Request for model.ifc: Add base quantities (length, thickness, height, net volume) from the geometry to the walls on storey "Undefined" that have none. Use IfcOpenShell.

First a look at what the model holds.

```python
import ifcopenshell
import ifcopenshell.util.element
import ifcopenshell.util.unit

model = ifcopenshell.open("model.ifc")
print(model.schema)
for unit_type in ("LENGTHUNIT", "AREAUNIT", "VOLUMEUNIT"):
    print(unit_type, ifcopenshell.util.unit.calculate_unit_scale(model, unit_type))
storey = next(s for s in model.by_type("IfcBuildingStorey") if s.Name == "Undefined")
walls = [e for e in ifcopenshell.util.element.get_decomposition(storey) if e.is_a("IfcWall")]
for e in sorted(walls, key=lambda e: e.id()):
    print(e.id(), e.is_a(), e.Name, list(ifcopenshell.util.element.get_psets(e, qtos_only=True)), sep=" | ")
```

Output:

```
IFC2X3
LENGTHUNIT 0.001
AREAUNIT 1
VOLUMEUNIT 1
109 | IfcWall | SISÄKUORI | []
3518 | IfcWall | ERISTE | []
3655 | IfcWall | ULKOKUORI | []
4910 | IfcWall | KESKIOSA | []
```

```python
import ifcopenshell
import ifcopenshell.api.pset
import ifcopenshell.geom
import ifcopenshell.util.element
import ifcopenshell.util.shape
import ifcopenshell.util.unit

model = ifcopenshell.open("model.ifc")
unit_scale = ifcopenshell.util.unit.calculate_unit_scale(model)
volume_scale = ifcopenshell.util.unit.calculate_unit_scale(model, "VOLUMEUNIT")
settings = ifcopenshell.geom.settings()

storey = next(s for s in model.by_type("IfcBuildingStorey") if s.Name == "Undefined")
walls = [e for e in ifcopenshell.util.element.get_decomposition(storey) if e.is_a("IfcWall")]

for e in sorted(walls, key=lambda e: e.id()):
    if ifcopenshell.util.element.get_psets(e, qtos_only=True, should_inherit=False):
        continue
    # Geometry comes back in metres, in the element's own axes.
    shape = ifcopenshell.geom.create_shape(settings, e)
    values = {
        "Length": ifcopenshell.util.shape.get_x(shape.geometry) / unit_scale,
        "Width": ifcopenshell.util.shape.get_y(shape.geometry) / unit_scale,
        "Height": ifcopenshell.util.shape.get_z(shape.geometry) / unit_scale,
        "NetVolume": ifcopenshell.util.shape.get_volume(shape.geometry) / volume_scale,
    }
    qto = ifcopenshell.api.pset.add_qto(model, product=e, name="BaseQuantities")
    ifcopenshell.api.pset.edit_qto(model, qto=qto, properties=values)
    print(e.id(), {k: round(v, 3) for k, v in values.items()})

model.write("model-out.ifc")
```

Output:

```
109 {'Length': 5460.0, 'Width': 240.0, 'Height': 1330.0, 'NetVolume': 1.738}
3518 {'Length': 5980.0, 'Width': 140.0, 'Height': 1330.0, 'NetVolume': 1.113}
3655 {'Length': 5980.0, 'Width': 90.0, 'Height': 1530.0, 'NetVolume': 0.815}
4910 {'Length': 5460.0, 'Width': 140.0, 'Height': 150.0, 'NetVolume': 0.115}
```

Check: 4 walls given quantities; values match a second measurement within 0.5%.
